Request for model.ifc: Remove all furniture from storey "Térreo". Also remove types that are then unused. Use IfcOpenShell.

First a look at what the model holds.

```python
import ifcopenshell
import ifcopenshell.util.element

model = ifcopenshell.open("model.ifc")
print(model.schema)
storey = next(s for s in model.by_type("IfcBuildingStorey") if s.Name == "Térreo")
furniture = [e for e in ifcopenshell.util.element.get_decomposition(storey) if e.is_a("IfcFurnishingElement")]
seen = {}
for e in furniture:
    element_type = ifcopenshell.util.element.get_type(e)
    name = element_type.Name if element_type not in (None, e) else None
    seen[name] = seen.get(name, 0) + 1
for name, count in sorted(seen.items(), key=str):
    print(count, "x", name)
```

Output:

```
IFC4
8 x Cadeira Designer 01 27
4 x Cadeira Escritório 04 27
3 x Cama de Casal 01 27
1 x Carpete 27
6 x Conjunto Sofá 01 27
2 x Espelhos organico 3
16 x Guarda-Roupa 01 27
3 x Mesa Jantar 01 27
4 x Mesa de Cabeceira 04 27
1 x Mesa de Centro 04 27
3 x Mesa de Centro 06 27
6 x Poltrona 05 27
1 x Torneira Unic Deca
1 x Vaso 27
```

```python
import ifcopenshell
import ifcopenshell.api.root
import ifcopenshell.util.element

model = ifcopenshell.open("model.ifc")

storey = next(s for s in model.by_type("IfcBuildingStorey") if s.Name == "Térreo")
furniture = [e for e in ifcopenshell.util.element.get_decomposition(storey) if e.is_a("IfcFurnishingElement")]
types = {ifcopenshell.util.element.get_type(e) for e in furniture} - {None, *furniture}

for e in furniture:
    ifcopenshell.api.root.remove_product(model, product=e)
print(len(furniture), "removed")

unused = [t for t in types if not ifcopenshell.util.element.get_types(t)]
for t in unused:
    ifcopenshell.api.root.remove_product(model, product=t)
print(len(unused), "unused types removed")

model.write("model-out.ifc")
```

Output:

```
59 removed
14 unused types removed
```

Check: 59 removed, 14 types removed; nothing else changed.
